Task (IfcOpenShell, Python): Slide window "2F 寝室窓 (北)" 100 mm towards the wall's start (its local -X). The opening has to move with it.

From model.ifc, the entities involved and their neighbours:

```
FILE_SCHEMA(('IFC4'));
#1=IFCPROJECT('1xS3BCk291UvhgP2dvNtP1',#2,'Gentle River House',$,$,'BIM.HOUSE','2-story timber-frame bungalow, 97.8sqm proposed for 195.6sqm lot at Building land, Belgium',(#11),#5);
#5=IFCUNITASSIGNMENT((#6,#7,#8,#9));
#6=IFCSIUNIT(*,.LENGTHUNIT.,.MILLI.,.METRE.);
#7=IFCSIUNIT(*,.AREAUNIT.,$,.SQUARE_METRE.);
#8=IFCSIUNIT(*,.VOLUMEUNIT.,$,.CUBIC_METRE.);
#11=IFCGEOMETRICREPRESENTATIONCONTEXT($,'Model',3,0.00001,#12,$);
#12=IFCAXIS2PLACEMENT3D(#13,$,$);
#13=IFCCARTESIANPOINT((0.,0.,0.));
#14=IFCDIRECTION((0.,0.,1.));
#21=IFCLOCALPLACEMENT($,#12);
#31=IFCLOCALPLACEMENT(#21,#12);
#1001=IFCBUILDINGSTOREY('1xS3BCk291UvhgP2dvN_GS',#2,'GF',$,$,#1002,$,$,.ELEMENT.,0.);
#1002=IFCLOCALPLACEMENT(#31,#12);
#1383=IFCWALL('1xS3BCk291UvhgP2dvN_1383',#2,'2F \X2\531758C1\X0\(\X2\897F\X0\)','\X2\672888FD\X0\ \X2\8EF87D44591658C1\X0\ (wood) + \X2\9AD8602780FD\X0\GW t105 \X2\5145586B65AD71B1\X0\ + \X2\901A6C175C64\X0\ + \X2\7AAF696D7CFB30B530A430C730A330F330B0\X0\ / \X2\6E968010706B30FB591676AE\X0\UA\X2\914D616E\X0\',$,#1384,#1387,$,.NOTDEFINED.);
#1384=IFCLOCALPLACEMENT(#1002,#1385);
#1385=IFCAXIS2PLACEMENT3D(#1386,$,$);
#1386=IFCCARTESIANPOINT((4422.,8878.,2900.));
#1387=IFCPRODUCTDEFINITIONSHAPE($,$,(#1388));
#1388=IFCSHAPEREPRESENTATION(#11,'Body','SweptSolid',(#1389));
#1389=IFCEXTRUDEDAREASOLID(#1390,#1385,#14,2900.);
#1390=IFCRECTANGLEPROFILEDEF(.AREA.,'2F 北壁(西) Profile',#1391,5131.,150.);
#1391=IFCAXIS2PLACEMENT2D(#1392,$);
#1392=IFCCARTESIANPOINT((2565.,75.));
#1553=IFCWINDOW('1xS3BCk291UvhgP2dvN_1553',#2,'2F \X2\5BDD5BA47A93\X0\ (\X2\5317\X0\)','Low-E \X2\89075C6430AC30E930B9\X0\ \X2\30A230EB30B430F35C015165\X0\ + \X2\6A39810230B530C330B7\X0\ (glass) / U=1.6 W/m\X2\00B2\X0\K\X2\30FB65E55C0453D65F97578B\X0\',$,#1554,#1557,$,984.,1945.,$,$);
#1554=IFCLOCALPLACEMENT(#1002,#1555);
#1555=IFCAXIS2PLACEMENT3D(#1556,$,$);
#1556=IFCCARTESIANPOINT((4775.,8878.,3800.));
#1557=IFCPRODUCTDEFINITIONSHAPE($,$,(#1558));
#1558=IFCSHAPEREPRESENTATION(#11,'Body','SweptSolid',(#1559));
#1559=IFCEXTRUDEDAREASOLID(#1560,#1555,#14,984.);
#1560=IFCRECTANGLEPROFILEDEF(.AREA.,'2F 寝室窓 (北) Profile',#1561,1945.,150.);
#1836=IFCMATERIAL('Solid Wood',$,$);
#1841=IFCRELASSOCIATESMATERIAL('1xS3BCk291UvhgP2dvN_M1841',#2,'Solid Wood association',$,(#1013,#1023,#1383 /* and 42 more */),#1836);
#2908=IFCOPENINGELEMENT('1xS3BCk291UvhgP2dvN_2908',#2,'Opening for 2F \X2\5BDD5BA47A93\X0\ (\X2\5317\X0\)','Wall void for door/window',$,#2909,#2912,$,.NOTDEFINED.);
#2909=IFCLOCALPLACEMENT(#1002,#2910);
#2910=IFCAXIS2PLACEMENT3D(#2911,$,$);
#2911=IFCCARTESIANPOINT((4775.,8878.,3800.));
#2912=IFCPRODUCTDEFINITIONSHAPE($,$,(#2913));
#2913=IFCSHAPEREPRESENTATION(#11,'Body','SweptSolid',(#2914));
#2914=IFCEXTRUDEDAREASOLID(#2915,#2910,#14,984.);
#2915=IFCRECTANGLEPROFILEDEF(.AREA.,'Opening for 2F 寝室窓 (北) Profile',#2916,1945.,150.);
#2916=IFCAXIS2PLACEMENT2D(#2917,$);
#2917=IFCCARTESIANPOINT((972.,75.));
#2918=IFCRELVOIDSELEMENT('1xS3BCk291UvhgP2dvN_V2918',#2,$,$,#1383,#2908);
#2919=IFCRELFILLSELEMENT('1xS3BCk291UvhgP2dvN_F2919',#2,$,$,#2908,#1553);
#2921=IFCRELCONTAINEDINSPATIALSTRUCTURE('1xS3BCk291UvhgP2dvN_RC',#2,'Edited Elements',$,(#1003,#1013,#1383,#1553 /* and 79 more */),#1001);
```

```python
import ifcopenshell
import ifcopenshell.api.geometry
import ifcopenshell.util.placement

model = ifcopenshell.open("model.ifc")

window = model.by_guid("1xS3BCk291UvhgP2dvN_1553")
opening = window.FillsVoids[0].RelatingOpeningElement
wall = opening.VoidsElements[0].RelatingBuildingElement

wall_matrix = ifcopenshell.util.placement.get_local_placement(wall.ObjectPlacement)
shift = wall_matrix[:3, 0] * -100.0
before = ifcopenshell.util.placement.get_local_placement(window.ObjectPlacement)[:3, 3].copy()

# The window is not placed relative to its opening, so move both.
for product in (opening, window):
    matrix = ifcopenshell.util.placement.get_local_placement(product.ObjectPlacement)
    matrix[:3, 3] += shift
    ifcopenshell.api.geometry.edit_object_placement(model, product=product, matrix=matrix, is_si=False)

after = ifcopenshell.util.placement.get_local_placement(window.ObjectPlacement)[:3, 3]
print("window moved by", (after - before).round(3) + 0.0)

model.write("model_updated.ifc")
```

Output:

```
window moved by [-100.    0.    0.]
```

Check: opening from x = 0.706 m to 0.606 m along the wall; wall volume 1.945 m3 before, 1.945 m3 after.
